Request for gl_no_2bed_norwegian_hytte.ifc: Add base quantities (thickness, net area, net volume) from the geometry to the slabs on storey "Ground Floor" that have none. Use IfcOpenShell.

First a look at what the model holds.

```python
import ifcopenshell
import ifcopenshell.util.element
import ifcopenshell.util.unit

model = ifcopenshell.open("gl_no_2bed_norwegian_hytte.ifc")
print(model.schema)
for unit_type in ("LENGTHUNIT", "AREAUNIT", "VOLUMEUNIT"):
    print(unit_type, ifcopenshell.util.unit.calculate_unit_scale(model, unit_type))
storey = next(s for s in model.by_type("IfcBuildingStorey") if s.Name == "Ground Floor")
slabs = [e for e in ifcopenshell.util.element.get_decomposition(storey) if e.is_a("IfcSlab")]
for e in sorted(slabs, key=lambda e: e.id()):
    print(e.id(), e.is_a(), e.Name, list(ifcopenshell.util.element.get_psets(e, qtos_only=True)), sep=" | ")
```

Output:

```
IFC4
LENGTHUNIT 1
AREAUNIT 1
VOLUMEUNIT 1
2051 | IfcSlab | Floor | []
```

```python
import ifcopenshell
import ifcopenshell.api.pset
import ifcopenshell.geom
import ifcopenshell.util.element
import ifcopenshell.util.shape
import ifcopenshell.util.unit

model = ifcopenshell.open("gl_no_2bed_norwegian_hytte.ifc")
unit_scale = ifcopenshell.util.unit.calculate_unit_scale(model)
area_scale = ifcopenshell.util.unit.calculate_unit_scale(model, "AREAUNIT")
volume_scale = ifcopenshell.util.unit.calculate_unit_scale(model, "VOLUMEUNIT")
settings = ifcopenshell.geom.settings()

storey = next(s for s in model.by_type("IfcBuildingStorey") if s.Name == "Ground Floor")
slabs = [e for e in ifcopenshell.util.element.get_decomposition(storey) if e.is_a("IfcSlab")]

for e in sorted(slabs, key=lambda e: e.id()):
    if ifcopenshell.util.element.get_psets(e, qtos_only=True, should_inherit=False):
        continue
    # Geometry comes back in metres, in the element's own axes.
    shape = ifcopenshell.geom.create_shape(settings, e)
    values = {
        "Width": ifcopenshell.util.shape.get_z(shape.geometry) / unit_scale,
        "NetArea": ifcopenshell.util.shape.get_footprint_area(shape.geometry) / area_scale,
        "NetVolume": ifcopenshell.util.shape.get_volume(shape.geometry) / volume_scale,
    }
    qto = ifcopenshell.api.pset.add_qto(model, product=e, name="Qto_SlabBaseQuantities")
    ifcopenshell.api.pset.edit_qto(model, qto=qto, properties=values)
    print(e.id(), {k: round(v, 3) for k, v in values.items()})

model.write("gl_no_2bed_norwegian_hytte_rev.ifc")
```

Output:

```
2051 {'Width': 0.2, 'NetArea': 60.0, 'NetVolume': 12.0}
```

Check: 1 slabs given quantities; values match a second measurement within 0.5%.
